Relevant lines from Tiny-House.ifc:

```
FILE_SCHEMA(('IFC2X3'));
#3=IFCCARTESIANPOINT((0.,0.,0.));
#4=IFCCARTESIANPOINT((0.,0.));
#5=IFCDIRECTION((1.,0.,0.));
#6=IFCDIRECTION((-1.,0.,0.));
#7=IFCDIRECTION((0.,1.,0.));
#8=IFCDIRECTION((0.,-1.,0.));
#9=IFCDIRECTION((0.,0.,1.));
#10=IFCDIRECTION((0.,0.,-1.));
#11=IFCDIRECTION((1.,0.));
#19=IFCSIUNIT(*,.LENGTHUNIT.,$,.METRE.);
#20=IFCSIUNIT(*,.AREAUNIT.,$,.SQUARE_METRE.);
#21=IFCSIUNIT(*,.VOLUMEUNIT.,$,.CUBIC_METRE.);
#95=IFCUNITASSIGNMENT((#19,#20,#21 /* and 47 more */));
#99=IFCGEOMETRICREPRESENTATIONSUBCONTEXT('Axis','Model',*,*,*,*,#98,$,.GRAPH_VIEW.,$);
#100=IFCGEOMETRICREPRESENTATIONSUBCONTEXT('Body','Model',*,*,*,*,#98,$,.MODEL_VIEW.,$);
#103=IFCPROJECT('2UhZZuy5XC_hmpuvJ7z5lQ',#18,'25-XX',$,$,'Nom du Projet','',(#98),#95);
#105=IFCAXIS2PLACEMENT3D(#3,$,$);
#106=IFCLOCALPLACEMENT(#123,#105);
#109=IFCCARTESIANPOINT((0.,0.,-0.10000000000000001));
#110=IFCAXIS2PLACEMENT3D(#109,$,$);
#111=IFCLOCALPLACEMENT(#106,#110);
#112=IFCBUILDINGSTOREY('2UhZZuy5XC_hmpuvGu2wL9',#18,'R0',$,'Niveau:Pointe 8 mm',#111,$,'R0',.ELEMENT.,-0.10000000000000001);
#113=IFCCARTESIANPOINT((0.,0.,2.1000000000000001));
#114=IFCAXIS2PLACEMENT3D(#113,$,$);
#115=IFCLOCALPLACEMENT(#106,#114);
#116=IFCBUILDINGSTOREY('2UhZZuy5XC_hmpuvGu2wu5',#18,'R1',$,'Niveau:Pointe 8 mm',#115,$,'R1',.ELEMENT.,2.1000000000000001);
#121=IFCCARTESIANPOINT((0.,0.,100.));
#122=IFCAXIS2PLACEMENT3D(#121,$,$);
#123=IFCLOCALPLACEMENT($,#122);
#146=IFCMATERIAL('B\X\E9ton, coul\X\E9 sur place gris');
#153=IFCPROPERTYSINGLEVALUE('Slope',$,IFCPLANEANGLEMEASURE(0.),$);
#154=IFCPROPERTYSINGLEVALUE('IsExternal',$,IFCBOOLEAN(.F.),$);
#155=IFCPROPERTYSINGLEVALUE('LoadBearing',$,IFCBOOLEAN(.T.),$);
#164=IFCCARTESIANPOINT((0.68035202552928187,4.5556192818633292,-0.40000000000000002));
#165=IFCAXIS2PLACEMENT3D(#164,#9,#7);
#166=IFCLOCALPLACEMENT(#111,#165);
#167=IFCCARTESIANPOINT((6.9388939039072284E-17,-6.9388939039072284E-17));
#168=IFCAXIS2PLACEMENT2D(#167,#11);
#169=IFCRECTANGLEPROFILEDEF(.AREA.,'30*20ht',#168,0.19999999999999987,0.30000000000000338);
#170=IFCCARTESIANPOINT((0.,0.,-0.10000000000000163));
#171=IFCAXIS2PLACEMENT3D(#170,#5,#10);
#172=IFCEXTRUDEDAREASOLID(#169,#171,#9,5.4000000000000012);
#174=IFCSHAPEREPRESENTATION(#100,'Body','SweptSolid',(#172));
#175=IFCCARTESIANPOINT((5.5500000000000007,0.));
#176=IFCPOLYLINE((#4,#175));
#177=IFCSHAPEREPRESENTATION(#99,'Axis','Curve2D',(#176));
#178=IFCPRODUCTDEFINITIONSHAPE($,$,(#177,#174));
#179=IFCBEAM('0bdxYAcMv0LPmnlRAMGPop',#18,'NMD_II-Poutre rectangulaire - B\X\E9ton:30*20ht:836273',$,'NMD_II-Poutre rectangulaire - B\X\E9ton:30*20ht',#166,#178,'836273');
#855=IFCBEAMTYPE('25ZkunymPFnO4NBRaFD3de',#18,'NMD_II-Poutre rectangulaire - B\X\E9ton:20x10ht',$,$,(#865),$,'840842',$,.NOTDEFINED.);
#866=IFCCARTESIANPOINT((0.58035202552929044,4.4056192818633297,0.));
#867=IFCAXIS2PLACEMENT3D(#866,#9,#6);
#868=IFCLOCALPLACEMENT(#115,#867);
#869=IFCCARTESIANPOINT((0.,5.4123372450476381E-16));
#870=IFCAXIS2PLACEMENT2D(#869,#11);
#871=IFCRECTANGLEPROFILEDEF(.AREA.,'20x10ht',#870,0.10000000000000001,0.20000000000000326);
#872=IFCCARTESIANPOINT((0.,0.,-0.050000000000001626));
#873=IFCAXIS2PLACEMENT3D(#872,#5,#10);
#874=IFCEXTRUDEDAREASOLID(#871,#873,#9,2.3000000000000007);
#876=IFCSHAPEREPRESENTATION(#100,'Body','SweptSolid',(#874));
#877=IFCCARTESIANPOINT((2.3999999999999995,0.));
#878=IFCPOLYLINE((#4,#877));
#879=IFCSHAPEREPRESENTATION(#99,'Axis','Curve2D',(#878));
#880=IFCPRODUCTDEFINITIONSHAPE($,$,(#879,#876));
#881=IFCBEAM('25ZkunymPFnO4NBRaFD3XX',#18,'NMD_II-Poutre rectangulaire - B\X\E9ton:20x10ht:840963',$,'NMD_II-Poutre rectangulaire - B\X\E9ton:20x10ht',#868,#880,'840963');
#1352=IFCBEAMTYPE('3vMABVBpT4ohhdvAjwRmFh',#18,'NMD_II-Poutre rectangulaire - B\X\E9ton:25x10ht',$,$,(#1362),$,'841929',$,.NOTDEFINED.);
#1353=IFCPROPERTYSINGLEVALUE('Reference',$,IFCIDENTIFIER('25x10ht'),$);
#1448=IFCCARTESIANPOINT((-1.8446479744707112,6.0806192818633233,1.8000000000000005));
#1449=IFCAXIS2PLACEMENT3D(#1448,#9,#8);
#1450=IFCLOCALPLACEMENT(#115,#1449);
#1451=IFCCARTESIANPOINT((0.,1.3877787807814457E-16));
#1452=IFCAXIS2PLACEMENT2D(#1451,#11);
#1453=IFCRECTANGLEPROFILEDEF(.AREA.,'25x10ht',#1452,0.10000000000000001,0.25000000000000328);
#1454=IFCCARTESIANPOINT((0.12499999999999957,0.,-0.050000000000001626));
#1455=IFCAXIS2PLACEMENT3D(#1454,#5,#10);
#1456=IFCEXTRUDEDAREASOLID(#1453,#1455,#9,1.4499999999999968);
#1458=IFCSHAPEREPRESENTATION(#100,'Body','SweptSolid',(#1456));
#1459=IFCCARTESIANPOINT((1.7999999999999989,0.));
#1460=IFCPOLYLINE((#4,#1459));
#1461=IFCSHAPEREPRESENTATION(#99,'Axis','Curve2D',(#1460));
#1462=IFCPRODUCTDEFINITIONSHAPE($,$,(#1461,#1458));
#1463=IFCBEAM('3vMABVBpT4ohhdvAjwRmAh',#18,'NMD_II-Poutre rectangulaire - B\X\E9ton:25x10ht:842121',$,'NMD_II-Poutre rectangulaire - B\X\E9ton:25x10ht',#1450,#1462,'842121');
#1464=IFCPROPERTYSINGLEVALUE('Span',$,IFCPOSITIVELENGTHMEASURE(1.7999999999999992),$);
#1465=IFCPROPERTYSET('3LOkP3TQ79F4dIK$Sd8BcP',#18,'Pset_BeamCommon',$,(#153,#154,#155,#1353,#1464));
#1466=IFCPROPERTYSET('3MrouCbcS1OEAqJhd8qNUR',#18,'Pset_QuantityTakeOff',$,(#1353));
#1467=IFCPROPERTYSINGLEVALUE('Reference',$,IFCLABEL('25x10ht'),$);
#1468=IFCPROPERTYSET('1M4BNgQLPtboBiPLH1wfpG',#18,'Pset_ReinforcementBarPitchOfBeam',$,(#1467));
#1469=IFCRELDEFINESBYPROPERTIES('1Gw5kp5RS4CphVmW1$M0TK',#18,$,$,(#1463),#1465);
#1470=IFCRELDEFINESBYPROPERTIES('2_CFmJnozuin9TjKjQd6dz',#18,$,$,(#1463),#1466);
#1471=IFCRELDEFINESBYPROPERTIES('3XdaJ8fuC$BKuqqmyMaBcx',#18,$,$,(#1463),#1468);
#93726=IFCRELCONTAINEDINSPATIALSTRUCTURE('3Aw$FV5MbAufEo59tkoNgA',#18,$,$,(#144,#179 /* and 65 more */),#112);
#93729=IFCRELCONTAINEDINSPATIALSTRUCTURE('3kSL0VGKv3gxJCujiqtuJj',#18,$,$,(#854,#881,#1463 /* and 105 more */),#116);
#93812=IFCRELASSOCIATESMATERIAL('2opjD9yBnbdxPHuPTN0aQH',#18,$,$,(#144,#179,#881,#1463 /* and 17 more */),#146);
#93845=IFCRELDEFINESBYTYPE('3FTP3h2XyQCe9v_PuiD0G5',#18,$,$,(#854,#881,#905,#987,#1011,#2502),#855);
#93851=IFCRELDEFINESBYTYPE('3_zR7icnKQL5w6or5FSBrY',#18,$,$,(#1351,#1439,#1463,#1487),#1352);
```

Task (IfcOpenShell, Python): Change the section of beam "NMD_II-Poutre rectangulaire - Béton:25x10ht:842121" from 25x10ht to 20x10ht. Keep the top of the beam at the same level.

```python
import ifcopenshell
import ifcopenshell.api.pset
import ifcopenshell.api.type
import ifcopenshell.util.element
import ifcopenshell.util.representation

model = ifcopenshell.open("Tiny-House.ifc")

member = model.by_guid("3vMABVBpT4ohhdvAjwRmAh")
source = next(p for p in model.by_type("IfcRectangleProfileDef") if p.ProfileName == "20x10ht")

body = ifcopenshell.util.representation.get_representation(member, "Model", "Body")
solid = body.Items[0]
old_profile = solid.SweptArea

# Copy the section's sizes but keep this member's own profile position.
profile = ifcopenshell.util.element.copy(model, source)
# Profiles are centred, so shift by half the change in depth to hold the top.
shift = (old_profile.XDim - profile.XDim) / 2
x, y = old_profile.Position.Location.Coordinates
up = (-1.0, 0.0)  # upwards, in the solid's own plane
location = model.createIfcCartesianPoint((x + up[0] * shift, y + up[1] * shift))
profile.Position = model.createIfcAxis2Placement2D(location, old_profile.Position.RefDirection)
solid.SweptArea = profile
if not model.get_total_inverses(old_profile):
    ifcopenshell.util.element.remove_deep2(model, old_profile)

new_type = model.by_id(855)
ifcopenshell.api.type.assign_type(
    model, related_objects=[member], relating_type=new_type, should_map_representations=False
)
member.Name = member.Name.replace("25x10ht", "20x10ht")
member.ObjectType = "NMD_II-Poutre rectangulaire - Béton:20x10ht"
pset = model.by_id(ifcopenshell.util.element.get_pset(member, "Pset_BeamCommon", should_inherit=False)["id"])
ifcopenshell.api.pset.edit_pset(model, pset=pset, properties={"Reference": "20x10ht"})
pset = model.by_id(ifcopenshell.util.element.get_pset(member, "Pset_QuantityTakeOff", should_inherit=False)["id"])
ifcopenshell.api.pset.edit_pset(model, pset=pset, properties={"Reference": "20x10ht"})
pset = model.by_id(ifcopenshell.util.element.get_pset(member, "Pset_ReinforcementBarPitchOfBeam", should_inherit=False)["id"])
ifcopenshell.api.pset.edit_pset(model, pset=pset, properties={"Reference": "20x10ht"})

print(solid.SweptArea)

model.write("Tiny-House_updated.ifc")
```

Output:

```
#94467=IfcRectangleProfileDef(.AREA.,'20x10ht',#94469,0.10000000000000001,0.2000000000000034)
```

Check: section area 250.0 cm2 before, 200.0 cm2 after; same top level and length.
